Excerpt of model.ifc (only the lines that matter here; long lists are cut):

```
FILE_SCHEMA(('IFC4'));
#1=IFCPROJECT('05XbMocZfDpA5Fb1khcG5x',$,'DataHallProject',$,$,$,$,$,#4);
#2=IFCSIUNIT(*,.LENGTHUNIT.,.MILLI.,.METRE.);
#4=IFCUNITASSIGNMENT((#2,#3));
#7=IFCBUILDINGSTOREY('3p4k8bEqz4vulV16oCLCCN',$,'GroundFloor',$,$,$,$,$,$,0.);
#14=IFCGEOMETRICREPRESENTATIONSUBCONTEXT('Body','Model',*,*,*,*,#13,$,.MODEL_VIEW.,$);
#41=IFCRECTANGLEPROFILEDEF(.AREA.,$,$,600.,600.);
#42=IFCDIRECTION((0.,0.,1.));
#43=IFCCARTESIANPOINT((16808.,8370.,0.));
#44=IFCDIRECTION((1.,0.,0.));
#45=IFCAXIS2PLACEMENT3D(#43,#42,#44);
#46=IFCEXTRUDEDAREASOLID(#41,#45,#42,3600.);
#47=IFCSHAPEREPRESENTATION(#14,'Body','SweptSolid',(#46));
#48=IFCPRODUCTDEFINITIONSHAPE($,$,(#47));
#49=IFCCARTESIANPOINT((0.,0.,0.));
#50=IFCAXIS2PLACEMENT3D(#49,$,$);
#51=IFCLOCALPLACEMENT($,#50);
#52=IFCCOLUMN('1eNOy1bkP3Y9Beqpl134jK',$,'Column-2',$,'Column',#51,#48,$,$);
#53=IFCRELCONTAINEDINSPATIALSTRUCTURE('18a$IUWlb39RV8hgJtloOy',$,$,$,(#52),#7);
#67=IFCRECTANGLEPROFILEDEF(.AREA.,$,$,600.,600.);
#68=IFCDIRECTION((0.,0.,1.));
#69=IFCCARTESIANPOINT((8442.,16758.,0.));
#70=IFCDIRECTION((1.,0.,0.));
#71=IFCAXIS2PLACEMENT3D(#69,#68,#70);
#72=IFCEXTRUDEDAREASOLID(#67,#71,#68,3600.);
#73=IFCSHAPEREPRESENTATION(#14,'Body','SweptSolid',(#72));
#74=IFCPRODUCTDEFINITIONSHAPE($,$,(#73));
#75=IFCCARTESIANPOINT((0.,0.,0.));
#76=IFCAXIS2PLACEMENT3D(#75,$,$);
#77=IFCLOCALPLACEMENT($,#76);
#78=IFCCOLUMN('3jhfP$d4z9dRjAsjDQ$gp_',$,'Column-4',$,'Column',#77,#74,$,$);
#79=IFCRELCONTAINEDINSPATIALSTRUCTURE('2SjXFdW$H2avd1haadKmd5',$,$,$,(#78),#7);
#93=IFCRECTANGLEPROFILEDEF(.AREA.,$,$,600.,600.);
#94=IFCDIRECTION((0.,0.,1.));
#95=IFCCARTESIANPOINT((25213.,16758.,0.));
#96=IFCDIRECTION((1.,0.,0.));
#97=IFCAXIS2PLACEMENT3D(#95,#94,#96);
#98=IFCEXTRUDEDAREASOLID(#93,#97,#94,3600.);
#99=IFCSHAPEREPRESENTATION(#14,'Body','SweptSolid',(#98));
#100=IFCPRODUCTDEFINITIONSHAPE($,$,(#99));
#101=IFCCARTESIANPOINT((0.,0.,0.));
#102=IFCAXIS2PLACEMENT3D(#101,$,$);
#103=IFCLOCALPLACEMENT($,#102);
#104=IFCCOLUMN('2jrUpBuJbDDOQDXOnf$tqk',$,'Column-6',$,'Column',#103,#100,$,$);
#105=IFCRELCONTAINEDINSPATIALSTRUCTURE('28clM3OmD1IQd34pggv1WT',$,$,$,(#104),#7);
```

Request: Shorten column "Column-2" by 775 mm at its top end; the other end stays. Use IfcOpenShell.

```python
import ifcopenshell
import ifcopenshell.util.representation

model = ifcopenshell.open("model.ifc")

member = model.by_id(52)
change = -775.0

# The extrusion runs towards the end named, so only its depth changes.
body = ifcopenshell.util.representation.get_representation(member, "Model", "Body")
solid = body.Items[0]
old_length = solid.Depth
solid.Depth += change

print(f"length {old_length:g} -> {solid.Depth:g}")

model.write("model_v2.ifc")
```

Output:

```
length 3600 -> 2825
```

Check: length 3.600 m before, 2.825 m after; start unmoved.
